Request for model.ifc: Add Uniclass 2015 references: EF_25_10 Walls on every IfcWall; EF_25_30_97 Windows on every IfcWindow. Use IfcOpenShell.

First a look at what the model holds.

```python
import ifcopenshell

model = ifcopenshell.open("model.ifc")
print(model.schema)
print("classifications:", [c.Name for c in model.by_type("IfcClassification")])
for ifc_class in ("IfcDoor", "IfcRoof", "IfcStair", "IfcWall", "IfcWindow"):
    print(ifc_class, len(model.by_type(ifc_class)))
```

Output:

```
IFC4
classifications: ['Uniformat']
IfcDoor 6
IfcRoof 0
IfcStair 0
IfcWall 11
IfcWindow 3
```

```python
import ifcopenshell
import ifcopenshell.api.classification

model = ifcopenshell.open("model.ifc")

system = ifcopenshell.api.classification.add_classification(model, classification="Uniclass 2015")

codes = {
    "IfcWall": ("EF_25_10", "Walls"),
    "IfcWindow": ("EF_25_30_97", "Windows"),
}
for ifc_class, (code, name) in codes.items():
    products = model.by_type(ifc_class)
    ifcopenshell.api.classification.add_reference(
        model, products=products, classification=system, identification=code, name=name
    )
    print(code, len(products))

model.write("model-out.ifc")
```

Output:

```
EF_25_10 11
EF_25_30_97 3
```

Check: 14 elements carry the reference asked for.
